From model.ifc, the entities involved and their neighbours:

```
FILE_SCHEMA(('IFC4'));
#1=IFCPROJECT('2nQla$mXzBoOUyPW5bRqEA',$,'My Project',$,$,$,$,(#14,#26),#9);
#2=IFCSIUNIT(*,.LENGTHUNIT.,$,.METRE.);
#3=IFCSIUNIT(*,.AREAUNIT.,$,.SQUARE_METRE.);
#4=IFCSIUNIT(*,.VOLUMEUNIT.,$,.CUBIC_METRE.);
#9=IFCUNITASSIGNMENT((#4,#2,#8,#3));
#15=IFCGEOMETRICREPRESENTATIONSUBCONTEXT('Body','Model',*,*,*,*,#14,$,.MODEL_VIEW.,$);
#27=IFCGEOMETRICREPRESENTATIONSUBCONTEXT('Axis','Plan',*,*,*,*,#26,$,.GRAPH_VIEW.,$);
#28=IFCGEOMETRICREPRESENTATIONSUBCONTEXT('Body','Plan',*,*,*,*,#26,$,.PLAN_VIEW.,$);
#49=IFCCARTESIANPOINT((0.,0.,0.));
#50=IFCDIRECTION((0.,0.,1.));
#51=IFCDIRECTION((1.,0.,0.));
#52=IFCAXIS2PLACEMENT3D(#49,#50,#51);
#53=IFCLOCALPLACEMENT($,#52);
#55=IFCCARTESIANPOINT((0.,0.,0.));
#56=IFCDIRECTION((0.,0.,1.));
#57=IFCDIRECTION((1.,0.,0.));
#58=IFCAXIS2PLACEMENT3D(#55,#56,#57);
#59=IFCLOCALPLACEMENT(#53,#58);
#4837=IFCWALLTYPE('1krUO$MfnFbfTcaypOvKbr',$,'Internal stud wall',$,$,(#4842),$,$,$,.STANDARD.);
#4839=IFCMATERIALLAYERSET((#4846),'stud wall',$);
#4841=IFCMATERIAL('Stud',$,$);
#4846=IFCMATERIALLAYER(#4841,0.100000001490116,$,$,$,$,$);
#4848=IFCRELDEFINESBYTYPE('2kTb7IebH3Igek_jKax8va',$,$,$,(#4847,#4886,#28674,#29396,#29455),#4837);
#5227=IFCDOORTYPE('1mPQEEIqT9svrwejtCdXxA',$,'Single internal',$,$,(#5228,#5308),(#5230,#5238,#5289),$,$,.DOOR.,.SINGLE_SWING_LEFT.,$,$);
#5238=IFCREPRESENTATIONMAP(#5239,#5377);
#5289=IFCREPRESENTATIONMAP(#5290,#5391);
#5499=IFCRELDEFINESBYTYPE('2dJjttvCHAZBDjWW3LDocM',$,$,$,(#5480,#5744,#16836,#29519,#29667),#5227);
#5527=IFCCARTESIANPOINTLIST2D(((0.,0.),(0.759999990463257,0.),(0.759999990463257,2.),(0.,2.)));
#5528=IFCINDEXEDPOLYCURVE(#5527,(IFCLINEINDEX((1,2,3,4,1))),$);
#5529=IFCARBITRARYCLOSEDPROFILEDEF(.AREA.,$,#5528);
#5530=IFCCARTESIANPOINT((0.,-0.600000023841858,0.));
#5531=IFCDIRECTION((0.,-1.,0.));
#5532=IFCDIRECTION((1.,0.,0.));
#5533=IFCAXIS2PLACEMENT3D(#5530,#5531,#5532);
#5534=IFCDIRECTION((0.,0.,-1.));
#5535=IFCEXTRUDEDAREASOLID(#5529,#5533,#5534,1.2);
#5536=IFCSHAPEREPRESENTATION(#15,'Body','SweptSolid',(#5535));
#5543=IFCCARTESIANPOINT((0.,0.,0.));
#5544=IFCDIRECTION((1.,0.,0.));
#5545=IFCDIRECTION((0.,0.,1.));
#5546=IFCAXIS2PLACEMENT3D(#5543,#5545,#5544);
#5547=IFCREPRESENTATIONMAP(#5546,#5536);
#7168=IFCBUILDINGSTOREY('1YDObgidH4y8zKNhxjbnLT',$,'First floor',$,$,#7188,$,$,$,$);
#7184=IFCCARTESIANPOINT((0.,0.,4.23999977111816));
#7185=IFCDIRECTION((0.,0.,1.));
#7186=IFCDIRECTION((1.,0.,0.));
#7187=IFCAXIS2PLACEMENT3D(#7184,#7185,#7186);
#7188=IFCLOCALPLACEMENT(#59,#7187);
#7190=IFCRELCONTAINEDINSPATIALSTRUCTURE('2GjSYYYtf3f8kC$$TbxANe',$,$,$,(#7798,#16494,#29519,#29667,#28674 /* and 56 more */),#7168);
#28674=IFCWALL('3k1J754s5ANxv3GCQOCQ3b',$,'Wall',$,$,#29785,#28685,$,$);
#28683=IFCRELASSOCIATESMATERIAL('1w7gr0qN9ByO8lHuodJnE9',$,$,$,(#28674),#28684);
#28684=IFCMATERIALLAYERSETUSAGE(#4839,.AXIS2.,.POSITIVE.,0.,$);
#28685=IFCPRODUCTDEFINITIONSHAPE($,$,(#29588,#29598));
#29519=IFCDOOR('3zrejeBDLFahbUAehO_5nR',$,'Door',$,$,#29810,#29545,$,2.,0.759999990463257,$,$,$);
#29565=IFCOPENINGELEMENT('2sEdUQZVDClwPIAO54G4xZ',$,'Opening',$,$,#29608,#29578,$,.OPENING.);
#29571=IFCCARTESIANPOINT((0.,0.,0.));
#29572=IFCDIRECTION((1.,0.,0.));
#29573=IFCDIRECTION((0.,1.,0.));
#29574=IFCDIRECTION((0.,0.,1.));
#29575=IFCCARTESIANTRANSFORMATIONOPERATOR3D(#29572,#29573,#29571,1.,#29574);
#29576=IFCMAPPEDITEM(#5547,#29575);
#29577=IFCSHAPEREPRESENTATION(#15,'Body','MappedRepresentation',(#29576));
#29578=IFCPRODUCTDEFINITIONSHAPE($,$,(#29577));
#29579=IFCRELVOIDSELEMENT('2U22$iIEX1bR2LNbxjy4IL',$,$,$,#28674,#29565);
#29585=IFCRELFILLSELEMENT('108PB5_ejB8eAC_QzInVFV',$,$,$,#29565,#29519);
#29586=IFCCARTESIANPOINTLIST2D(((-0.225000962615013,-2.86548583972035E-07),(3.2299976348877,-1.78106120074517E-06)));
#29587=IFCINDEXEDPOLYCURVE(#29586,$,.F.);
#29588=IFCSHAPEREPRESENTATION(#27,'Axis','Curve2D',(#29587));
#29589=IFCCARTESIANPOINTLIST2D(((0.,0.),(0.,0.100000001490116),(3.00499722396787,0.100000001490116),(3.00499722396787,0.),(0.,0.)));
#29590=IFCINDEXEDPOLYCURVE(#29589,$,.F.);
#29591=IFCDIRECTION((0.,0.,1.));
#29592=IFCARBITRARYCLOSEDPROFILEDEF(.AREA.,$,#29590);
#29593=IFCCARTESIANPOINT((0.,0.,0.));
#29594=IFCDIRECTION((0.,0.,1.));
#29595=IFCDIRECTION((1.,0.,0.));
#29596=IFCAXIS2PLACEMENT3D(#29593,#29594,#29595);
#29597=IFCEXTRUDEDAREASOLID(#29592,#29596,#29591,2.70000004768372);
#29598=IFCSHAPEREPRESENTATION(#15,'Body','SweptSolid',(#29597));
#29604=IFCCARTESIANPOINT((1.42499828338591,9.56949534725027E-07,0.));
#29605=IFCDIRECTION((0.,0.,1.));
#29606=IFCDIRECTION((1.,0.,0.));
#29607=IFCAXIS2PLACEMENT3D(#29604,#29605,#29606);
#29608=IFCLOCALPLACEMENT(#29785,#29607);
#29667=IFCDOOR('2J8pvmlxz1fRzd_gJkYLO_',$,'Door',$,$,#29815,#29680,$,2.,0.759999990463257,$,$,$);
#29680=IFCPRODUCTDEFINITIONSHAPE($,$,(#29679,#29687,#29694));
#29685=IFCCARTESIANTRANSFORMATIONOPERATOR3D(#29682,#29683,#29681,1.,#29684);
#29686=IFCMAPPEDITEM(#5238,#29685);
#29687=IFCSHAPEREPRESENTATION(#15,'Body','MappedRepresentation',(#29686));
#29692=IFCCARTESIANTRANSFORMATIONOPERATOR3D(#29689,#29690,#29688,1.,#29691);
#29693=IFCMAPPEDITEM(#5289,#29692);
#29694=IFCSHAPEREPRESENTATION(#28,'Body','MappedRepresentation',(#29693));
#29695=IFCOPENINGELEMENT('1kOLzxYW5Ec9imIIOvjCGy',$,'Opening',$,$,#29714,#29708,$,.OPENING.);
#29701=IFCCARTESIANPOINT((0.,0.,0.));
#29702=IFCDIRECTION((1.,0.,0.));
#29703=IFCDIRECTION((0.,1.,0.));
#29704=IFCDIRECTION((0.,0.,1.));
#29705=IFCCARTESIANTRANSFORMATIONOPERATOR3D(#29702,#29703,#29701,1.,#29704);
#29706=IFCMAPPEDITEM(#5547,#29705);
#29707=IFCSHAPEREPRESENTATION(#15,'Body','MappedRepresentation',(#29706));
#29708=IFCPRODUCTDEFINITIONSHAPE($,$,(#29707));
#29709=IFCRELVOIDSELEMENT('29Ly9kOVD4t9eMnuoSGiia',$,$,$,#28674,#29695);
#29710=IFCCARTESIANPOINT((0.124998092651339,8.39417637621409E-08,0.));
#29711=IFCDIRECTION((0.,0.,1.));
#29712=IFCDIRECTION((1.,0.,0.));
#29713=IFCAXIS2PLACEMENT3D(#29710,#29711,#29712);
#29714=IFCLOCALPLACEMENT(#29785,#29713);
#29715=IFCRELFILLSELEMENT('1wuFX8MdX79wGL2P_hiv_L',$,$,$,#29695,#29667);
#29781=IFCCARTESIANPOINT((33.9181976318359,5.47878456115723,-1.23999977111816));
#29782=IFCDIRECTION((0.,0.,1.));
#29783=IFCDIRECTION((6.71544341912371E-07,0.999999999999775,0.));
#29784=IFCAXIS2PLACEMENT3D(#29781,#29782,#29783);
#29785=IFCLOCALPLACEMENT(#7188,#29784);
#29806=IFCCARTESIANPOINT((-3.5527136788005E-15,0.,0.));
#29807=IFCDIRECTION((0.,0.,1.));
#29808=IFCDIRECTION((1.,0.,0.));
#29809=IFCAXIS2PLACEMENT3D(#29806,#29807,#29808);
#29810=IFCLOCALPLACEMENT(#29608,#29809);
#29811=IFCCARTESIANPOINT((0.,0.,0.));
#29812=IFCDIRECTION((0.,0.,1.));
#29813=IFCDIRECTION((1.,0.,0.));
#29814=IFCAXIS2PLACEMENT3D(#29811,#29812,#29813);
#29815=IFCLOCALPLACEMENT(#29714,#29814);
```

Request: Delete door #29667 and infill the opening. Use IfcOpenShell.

```python
import ifcopenshell
import ifcopenshell.api.feature
import ifcopenshell.api.root
import ifcopenshell.geom
import ifcopenshell.util.shape

model = ifcopenshell.open("model.ifc")
settings = ifcopenshell.geom.settings()


def volume(element):
    """Net volume in cubic metres, openings subtracted."""
    shape = ifcopenshell.geom.create_shape(settings, element)
    return ifcopenshell.util.shape.get_volume(shape.geometry)


door = model.by_guid("2J8pvmlxz1fRzd_gJkYLO_")
opening = door.FillsVoids[0].RelatingOpeningElement
wall = opening.VoidsElements[0].RelatingBuildingElement
before = volume(wall)

ifcopenshell.api.root.remove_product(model, product=door)
ifcopenshell.api.feature.remove_feature(model, feature=opening)

after = volume(wall)

print(f"wall volume {before:.3f} -> {after:.3f} m3")

model.write("model_rev.ifc")
```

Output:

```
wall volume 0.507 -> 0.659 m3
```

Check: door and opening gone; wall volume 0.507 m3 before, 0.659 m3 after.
